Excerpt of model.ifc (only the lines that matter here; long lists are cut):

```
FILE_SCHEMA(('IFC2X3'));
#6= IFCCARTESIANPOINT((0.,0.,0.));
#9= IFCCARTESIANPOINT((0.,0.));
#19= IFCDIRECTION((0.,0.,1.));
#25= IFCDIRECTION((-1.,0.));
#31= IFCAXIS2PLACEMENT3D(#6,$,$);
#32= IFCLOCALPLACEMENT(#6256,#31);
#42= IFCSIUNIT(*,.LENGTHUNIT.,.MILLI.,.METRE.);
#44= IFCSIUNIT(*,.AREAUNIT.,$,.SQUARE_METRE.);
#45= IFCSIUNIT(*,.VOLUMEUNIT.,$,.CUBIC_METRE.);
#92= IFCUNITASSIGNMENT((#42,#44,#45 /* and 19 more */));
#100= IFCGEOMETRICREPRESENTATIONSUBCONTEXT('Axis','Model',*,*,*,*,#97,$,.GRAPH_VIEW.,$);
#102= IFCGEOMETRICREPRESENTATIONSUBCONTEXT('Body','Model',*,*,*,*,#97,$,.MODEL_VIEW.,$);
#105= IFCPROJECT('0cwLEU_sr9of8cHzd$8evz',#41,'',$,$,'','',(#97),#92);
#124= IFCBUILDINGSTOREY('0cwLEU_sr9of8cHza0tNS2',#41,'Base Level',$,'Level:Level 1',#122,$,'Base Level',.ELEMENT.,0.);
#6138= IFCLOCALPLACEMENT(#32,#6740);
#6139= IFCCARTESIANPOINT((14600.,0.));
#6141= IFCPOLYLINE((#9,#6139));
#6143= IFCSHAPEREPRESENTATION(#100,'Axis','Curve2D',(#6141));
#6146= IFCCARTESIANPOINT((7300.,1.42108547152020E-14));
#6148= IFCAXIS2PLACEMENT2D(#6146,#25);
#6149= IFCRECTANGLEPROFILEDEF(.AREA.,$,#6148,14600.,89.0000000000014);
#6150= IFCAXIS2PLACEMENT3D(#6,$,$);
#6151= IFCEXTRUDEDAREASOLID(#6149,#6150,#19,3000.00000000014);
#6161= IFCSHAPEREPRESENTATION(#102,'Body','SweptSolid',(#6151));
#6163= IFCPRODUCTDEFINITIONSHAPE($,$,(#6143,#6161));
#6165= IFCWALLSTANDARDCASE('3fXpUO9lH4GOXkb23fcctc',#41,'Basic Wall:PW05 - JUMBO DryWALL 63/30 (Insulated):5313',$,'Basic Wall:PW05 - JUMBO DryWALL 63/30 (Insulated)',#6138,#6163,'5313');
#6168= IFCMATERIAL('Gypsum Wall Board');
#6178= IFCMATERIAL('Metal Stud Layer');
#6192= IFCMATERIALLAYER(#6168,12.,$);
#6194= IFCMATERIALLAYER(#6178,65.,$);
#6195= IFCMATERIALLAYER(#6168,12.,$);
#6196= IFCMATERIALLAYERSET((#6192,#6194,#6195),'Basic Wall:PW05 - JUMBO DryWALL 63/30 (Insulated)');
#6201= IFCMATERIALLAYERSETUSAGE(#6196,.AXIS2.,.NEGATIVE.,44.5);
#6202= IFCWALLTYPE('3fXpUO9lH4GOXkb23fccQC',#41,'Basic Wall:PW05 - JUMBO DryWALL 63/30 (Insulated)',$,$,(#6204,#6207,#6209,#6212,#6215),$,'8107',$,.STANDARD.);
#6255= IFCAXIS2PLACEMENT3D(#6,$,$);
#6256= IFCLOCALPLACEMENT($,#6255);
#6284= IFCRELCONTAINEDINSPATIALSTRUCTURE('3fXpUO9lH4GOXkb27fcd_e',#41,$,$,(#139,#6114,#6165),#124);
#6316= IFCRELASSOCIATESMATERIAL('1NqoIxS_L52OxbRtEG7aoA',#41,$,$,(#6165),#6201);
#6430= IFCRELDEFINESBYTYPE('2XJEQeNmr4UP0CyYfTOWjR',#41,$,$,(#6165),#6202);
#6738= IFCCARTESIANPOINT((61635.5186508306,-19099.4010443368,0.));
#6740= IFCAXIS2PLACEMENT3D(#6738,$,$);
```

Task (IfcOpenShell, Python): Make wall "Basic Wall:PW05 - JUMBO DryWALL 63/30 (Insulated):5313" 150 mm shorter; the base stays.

```python
import ifcopenshell
import ifcopenshell.geom
import ifcopenshell.util.representation
import ifcopenshell.util.shape
import ifcopenshell.util.unit

model = ifcopenshell.open("model.ifc")
unit_scale = ifcopenshell.util.unit.calculate_unit_scale(model)
settings = ifcopenshell.geom.settings()


def volume(element):
    """Net volume in cubic metres, openings subtracted."""
    shape = ifcopenshell.geom.create_shape(settings, element)
    return ifcopenshell.util.shape.get_volume(shape.geometry)


wall = model.by_guid("3fXpUO9lH4GOXkb23fcctc")
before = volume(wall)

body = ifcopenshell.util.representation.get_representation(wall, "Model", "Body")
solid = body.Items[0]
old_height = solid.Depth
solid.Depth -= 0.15 / unit_scale
after = volume(wall)

print(f"height {old_height:g} -> {solid.Depth:g}, volume {before:.3f} -> {after:.3f} m3")

model.write("model_edited.ifc")
```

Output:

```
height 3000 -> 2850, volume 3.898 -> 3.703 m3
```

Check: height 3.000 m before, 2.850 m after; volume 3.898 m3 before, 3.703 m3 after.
